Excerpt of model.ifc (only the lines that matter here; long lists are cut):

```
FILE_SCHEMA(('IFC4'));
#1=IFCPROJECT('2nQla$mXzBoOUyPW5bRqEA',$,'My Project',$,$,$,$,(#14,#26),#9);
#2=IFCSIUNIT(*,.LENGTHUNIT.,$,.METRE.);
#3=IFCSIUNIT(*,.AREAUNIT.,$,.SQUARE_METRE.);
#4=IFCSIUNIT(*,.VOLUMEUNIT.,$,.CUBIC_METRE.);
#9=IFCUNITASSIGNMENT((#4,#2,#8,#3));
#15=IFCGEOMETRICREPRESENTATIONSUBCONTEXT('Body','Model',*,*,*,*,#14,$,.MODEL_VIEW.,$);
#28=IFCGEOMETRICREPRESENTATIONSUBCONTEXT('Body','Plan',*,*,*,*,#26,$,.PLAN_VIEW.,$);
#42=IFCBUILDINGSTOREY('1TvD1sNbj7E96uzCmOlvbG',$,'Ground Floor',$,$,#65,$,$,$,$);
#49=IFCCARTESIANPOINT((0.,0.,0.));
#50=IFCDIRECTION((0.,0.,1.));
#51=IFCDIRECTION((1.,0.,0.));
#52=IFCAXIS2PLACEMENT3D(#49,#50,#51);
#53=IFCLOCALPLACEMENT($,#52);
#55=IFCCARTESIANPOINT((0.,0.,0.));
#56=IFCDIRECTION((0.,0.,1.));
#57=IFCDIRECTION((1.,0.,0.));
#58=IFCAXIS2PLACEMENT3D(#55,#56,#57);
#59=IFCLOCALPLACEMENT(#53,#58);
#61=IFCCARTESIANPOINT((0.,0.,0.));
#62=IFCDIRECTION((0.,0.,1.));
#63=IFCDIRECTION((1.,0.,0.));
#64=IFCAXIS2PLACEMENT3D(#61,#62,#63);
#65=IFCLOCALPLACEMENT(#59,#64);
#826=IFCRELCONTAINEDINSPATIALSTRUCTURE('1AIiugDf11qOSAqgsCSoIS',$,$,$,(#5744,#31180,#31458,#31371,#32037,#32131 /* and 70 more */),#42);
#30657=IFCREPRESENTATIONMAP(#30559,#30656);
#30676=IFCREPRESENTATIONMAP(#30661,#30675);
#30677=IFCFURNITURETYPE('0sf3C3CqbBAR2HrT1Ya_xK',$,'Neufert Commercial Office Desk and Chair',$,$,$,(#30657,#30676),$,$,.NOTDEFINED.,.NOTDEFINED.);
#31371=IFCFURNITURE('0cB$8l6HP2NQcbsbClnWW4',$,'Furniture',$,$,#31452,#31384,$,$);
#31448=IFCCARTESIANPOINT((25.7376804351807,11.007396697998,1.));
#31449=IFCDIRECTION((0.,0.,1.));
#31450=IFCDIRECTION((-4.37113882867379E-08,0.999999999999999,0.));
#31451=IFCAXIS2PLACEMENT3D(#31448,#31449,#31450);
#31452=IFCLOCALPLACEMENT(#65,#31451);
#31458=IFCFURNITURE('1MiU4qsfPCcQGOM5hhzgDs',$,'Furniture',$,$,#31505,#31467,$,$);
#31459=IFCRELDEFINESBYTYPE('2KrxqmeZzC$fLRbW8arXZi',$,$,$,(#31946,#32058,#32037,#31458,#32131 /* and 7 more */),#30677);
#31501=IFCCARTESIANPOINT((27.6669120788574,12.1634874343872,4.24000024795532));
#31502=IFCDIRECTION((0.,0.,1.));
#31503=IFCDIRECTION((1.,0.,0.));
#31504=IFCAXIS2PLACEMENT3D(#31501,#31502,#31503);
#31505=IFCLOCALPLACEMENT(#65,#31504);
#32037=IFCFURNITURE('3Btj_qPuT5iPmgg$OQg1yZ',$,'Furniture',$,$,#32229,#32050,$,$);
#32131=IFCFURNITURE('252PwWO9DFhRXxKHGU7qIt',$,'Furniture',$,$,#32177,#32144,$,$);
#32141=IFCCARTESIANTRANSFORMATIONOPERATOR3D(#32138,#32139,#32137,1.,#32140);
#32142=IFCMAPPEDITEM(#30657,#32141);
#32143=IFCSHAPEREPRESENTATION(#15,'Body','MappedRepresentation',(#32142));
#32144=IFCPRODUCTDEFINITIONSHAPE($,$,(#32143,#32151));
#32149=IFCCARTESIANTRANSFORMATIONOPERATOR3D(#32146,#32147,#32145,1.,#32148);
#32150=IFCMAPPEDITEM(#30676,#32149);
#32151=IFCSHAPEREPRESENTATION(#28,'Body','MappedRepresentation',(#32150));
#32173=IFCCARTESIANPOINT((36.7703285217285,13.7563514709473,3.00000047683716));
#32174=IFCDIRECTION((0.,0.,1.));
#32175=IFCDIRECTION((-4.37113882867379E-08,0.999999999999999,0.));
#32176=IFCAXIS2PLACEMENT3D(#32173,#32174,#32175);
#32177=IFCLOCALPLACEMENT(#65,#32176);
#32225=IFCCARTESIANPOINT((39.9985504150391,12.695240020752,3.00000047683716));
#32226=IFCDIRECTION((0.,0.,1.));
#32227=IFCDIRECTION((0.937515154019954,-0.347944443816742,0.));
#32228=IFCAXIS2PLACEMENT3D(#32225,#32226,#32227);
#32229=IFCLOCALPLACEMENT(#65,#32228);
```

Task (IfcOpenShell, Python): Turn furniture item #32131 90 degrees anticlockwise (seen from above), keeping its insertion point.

```python
import ifcopenshell
import ifcopenshell.api.geometry
import ifcopenshell.util.placement

model = ifcopenshell.open("model.ifc")

item = model.by_guid("252PwWO9DFhRXxKHGU7qIt")
matrix = ifcopenshell.util.placement.get_local_placement(item.ObjectPlacement)
matrix = matrix @ ifcopenshell.util.placement.rotation(90, "Z")
ifcopenshell.api.geometry.edit_object_placement(model, product=item, matrix=matrix, is_si=False)

print(ifcopenshell.util.placement.get_local_placement(item.ObjectPlacement).round(3) + 0.0)

model.write("model_updated.ifc")
```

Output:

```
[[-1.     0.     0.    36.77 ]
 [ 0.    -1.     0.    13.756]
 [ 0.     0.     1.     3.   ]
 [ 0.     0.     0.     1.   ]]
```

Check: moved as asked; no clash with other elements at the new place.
